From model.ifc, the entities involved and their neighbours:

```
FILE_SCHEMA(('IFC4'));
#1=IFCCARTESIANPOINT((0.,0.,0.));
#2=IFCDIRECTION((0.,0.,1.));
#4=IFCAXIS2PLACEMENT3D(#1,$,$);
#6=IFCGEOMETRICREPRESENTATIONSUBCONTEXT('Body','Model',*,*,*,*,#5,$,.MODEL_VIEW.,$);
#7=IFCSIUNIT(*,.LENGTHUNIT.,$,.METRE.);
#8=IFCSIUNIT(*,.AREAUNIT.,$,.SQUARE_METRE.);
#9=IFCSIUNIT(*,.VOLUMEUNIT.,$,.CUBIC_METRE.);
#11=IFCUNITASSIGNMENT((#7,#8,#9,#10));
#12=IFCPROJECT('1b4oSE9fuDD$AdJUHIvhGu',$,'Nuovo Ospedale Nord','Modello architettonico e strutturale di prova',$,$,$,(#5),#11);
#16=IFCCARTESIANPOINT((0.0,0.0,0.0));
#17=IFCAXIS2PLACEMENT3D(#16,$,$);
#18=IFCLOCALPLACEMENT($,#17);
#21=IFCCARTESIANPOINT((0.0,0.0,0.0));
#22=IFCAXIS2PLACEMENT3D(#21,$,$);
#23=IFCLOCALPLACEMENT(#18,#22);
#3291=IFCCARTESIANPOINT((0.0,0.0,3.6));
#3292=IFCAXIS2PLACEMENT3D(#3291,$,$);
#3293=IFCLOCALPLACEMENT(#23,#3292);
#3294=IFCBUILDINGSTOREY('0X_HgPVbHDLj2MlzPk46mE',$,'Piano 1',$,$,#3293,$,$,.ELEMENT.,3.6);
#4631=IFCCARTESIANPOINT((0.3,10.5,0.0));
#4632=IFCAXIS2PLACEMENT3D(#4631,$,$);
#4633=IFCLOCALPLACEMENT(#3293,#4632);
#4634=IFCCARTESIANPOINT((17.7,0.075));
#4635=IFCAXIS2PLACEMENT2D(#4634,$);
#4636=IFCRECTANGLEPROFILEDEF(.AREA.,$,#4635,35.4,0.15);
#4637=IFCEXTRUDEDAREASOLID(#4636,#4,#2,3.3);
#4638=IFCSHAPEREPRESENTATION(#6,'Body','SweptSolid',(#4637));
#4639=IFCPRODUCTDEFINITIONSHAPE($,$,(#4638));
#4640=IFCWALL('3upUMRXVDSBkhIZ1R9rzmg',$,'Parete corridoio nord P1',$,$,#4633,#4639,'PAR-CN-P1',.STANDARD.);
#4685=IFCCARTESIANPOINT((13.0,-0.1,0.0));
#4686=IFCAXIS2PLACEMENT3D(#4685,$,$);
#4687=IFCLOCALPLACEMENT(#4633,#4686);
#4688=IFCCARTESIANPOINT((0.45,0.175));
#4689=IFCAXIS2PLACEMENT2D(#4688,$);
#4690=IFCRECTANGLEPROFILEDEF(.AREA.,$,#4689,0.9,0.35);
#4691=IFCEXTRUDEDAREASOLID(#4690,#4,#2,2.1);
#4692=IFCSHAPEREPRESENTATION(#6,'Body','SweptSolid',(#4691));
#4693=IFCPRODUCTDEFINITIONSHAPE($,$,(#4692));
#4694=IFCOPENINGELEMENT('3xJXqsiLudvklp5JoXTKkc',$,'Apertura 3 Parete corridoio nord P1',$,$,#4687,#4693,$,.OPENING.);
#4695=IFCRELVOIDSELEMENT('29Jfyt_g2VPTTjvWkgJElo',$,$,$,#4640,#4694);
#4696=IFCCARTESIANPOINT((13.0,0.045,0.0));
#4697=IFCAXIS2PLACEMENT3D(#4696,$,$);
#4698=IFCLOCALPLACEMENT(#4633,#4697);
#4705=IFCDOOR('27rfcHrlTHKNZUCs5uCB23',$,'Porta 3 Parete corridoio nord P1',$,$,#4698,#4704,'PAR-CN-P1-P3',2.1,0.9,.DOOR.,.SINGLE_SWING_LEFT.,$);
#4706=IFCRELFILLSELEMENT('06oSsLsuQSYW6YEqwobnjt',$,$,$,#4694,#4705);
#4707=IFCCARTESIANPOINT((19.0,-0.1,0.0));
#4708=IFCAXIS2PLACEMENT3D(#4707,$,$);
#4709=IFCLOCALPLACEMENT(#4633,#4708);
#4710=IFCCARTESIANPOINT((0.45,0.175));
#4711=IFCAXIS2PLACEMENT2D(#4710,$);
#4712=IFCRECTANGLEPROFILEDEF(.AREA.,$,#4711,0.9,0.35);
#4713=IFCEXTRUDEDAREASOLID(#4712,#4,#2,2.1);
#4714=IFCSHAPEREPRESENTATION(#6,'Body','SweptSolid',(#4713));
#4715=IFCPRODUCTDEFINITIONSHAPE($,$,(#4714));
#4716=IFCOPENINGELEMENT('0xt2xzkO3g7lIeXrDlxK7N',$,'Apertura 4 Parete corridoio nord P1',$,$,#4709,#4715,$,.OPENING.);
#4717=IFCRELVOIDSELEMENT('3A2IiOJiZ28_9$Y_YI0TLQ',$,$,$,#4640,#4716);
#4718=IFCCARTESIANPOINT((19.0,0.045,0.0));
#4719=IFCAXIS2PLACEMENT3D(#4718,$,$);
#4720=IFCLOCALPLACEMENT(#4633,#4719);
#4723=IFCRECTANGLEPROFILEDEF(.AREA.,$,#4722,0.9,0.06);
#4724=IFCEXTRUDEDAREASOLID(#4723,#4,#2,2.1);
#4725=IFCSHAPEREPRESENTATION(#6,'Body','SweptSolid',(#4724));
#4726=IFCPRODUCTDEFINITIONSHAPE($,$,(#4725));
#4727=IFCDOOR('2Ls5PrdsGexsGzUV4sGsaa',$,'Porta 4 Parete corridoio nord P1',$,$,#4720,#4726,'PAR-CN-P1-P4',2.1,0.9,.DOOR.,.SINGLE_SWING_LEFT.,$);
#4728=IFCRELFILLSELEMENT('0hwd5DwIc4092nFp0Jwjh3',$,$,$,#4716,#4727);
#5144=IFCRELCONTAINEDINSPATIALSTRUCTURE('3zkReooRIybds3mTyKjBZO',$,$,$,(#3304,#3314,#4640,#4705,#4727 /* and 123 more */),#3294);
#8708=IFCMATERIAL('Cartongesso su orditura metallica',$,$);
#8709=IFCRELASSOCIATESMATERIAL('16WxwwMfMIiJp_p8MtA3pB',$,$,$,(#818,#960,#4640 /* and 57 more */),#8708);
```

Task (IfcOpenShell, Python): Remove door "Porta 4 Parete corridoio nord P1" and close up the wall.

```python
import ifcopenshell
import ifcopenshell.api.feature
import ifcopenshell.api.root
import ifcopenshell.geom
import ifcopenshell.util.shape

model = ifcopenshell.open("model.ifc")
settings = ifcopenshell.geom.settings()


def volume(element):
    """Net volume in cubic metres, openings subtracted."""
    shape = ifcopenshell.geom.create_shape(settings, element)
    return ifcopenshell.util.shape.get_volume(shape.geometry)


door = model.by_guid("2Ls5PrdsGexsGzUV4sGsaa")
opening = door.FillsVoids[0].RelatingOpeningElement
wall = opening.VoidsElements[0].RelatingBuildingElement
before = volume(wall)

ifcopenshell.api.root.remove_product(model, product=door)
ifcopenshell.api.feature.remove_feature(model, feature=opening)

after = volume(wall)

print(f"wall volume {before:.3f} -> {after:.3f} m3")

model.write("model_updated.ifc")
```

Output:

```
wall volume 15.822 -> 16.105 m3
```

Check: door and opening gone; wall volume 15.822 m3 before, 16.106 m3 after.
